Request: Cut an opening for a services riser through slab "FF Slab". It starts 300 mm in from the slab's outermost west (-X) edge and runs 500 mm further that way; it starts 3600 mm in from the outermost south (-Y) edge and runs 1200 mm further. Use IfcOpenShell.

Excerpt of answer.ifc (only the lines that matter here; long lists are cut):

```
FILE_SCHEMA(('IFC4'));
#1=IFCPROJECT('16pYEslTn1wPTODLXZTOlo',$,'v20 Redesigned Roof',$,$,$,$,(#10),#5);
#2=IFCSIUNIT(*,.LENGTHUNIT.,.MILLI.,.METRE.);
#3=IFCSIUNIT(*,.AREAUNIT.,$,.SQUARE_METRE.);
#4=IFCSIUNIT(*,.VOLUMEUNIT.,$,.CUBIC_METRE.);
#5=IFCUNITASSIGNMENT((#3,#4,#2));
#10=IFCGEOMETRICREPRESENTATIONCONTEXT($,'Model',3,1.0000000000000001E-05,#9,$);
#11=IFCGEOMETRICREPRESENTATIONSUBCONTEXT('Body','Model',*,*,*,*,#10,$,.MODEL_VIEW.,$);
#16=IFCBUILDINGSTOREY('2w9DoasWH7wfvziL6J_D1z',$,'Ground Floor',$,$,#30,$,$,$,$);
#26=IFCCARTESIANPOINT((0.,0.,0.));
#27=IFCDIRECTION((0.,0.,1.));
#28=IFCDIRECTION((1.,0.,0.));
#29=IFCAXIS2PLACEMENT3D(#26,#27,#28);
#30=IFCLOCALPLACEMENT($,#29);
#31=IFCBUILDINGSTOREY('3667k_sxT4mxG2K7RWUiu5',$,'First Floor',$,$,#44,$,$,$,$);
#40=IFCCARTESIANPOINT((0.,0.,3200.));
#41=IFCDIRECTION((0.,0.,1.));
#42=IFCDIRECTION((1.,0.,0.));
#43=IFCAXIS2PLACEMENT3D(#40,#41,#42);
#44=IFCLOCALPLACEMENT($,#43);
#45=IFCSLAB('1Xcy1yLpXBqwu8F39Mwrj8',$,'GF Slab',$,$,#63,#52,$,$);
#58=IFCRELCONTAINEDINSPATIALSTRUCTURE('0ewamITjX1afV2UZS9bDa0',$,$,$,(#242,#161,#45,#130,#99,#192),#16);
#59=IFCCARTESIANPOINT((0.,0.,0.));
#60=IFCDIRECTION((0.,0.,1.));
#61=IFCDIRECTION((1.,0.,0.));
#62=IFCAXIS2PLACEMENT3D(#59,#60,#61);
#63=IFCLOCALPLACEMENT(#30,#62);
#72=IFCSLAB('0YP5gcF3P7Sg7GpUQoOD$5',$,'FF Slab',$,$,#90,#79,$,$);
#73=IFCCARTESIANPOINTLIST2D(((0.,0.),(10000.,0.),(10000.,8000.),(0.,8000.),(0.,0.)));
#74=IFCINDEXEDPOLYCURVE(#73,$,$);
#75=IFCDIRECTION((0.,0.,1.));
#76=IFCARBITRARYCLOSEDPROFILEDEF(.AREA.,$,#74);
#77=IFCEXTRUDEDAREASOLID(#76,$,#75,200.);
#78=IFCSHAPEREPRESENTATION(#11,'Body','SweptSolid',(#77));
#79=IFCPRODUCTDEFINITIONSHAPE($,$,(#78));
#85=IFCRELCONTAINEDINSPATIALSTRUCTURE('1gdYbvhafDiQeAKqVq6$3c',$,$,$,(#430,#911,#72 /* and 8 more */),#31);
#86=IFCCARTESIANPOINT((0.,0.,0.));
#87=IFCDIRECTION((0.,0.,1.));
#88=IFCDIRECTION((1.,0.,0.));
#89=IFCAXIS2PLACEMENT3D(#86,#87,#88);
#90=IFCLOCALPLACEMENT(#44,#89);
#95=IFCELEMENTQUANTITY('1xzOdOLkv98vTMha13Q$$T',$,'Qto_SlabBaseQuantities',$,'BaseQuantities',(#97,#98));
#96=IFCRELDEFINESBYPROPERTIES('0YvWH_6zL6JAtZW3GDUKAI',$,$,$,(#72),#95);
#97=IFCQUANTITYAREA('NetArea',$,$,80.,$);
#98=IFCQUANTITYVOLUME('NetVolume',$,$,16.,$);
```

```python
import numpy as np
import ifcopenshell
import ifcopenshell.api.feature
import ifcopenshell.api.geometry
import ifcopenshell.api.pset
import ifcopenshell.api.root
import ifcopenshell.geom
import ifcopenshell.util.element
import ifcopenshell.util.placement
import ifcopenshell.util.representation
import ifcopenshell.util.shape
import ifcopenshell.util.unit

model = ifcopenshell.open("answer.ifc")
unit_scale = ifcopenshell.util.unit.calculate_unit_scale(model)
area_scale = ifcopenshell.util.unit.calculate_unit_scale(model, "AREAUNIT")
volume_scale = ifcopenshell.util.unit.calculate_unit_scale(model, "VOLUMEUNIT")
settings = ifcopenshell.geom.settings()


def volume(element):
    """Net volume in cubic metres, openings subtracted."""
    shape = ifcopenshell.geom.create_shape(settings, element)
    return ifcopenshell.util.shape.get_volume(shape.geometry)


slab = model.by_id(72)
before = volume(slab)

# Extent in the slab's own axes, in metres. The edges named are its -X and -Y sides.
slab_shape = ifcopenshell.geom.create_shape(settings, slab)
vertices = ifcopenshell.util.shape.get_vertices(slab_shape.geometry)
x_min, y_min, bottom = vertices.min(axis=0)
top = vertices[:, 2].max()

opening = ifcopenshell.api.root.create_entity(model, ifc_class="IfcOpeningElement", name="Services riser opening", predefined_type="OPENING")
context = ifcopenshell.util.representation.get_context(model, "Model", "Body", "MODEL_VIEW")
width, depth = 0.5, 1.2
outline = [(0.0, 0.0), (width, 0.0), (width, depth), (0.0, depth), (0.0, 0.0)]
# Overshoot both faces by 50 mm so the cut is clean.
shape = ifcopenshell.api.geometry.add_slab_representation(
    model, context=context, depth=top - bottom + 0.1, polyline=outline
)
ifcopenshell.api.geometry.assign_representation(model, product=opening, representation=shape)

matrix = ifcopenshell.util.placement.get_local_placement(slab.ObjectPlacement)
matrix[:, 3] = matrix @ np.append(np.array([x_min + 0.3, y_min + 3.6, bottom - 0.05]) / unit_scale, 1.0)
ifcopenshell.api.geometry.edit_object_placement(model, product=opening, matrix=matrix, is_si=False)
ifcopenshell.api.feature.add_feature(model, feature=opening, element=slab)

after = volume(slab)

# Update the slab's stored quantities.
qto = model.by_id(ifcopenshell.util.element.get_pset(slab, "Qto_SlabBaseQuantities", should_inherit=False)["id"])
ifcopenshell.api.pset.edit_qto(model, qto=qto, properties={
    "NetArea": after / (top - bottom) / area_scale,
    "NetVolume": after / volume_scale,
})

print(f"slab volume {before:.3f} -> {after:.3f} m3")

model.write("answer_v2.ifc")
```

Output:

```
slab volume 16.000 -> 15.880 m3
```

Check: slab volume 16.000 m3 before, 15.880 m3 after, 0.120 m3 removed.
